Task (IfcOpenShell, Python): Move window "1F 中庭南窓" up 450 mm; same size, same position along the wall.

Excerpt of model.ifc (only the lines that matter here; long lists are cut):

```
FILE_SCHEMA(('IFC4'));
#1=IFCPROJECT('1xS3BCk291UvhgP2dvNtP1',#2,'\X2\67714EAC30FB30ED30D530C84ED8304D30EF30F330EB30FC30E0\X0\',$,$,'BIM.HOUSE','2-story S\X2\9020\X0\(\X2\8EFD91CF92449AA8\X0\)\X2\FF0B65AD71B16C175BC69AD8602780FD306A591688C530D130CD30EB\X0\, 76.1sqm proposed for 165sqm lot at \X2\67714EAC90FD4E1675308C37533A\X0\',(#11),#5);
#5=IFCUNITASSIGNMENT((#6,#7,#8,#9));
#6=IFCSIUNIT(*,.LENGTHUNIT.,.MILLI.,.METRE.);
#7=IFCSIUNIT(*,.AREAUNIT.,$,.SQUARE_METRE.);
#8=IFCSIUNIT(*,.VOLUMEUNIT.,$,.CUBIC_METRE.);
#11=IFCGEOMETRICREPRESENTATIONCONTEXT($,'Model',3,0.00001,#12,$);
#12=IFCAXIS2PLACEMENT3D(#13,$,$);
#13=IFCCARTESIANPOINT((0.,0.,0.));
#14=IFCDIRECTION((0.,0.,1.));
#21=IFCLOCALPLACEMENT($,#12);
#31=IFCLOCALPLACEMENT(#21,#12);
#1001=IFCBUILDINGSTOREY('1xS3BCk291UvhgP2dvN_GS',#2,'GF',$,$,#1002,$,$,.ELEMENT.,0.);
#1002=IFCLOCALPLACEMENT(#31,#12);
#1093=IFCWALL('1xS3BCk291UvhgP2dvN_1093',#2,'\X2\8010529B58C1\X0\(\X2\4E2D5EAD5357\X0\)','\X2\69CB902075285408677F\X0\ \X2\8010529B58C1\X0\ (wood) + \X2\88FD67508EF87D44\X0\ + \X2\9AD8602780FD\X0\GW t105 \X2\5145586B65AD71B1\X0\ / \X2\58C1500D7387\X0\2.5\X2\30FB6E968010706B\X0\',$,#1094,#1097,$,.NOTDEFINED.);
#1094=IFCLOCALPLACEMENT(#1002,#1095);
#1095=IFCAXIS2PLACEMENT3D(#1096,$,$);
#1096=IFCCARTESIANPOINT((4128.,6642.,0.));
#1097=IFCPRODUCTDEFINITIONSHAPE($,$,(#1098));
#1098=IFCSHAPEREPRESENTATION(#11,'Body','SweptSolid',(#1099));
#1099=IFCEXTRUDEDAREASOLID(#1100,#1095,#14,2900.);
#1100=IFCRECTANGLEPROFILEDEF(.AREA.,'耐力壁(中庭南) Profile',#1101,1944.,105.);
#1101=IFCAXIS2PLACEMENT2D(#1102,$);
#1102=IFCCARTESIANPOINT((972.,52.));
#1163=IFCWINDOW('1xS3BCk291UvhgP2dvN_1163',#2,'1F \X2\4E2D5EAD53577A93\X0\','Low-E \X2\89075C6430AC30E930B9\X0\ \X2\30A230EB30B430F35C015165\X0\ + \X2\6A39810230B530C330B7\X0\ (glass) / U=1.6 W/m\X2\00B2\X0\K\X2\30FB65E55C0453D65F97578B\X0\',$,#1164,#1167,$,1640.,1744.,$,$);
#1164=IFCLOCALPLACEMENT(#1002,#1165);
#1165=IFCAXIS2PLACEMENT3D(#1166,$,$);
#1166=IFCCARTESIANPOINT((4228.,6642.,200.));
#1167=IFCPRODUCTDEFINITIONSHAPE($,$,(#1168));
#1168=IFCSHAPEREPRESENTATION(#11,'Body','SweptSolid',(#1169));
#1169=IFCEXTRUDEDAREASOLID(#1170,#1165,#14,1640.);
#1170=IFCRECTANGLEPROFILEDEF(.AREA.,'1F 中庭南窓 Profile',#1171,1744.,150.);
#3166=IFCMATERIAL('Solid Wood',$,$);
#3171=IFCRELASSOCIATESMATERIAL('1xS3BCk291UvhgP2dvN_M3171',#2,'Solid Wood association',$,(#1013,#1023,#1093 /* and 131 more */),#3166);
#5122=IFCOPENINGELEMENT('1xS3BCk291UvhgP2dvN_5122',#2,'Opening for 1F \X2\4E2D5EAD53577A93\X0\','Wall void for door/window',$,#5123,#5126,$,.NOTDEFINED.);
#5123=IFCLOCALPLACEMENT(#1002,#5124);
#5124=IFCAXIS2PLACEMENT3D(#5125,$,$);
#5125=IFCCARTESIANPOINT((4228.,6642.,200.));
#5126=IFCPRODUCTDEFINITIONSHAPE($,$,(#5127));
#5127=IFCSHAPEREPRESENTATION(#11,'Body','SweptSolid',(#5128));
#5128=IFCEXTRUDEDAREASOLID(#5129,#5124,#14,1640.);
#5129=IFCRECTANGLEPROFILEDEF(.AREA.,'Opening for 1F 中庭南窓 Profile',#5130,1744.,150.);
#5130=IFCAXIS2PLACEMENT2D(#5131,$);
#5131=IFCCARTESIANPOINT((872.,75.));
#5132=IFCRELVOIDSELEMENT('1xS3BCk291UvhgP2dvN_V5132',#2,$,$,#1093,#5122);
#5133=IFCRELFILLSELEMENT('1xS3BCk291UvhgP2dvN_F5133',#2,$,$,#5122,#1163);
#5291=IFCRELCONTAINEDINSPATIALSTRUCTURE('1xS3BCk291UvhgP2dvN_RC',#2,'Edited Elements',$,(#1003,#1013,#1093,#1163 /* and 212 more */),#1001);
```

```python
import numpy as np
import ifcopenshell
import ifcopenshell.api.geometry
import ifcopenshell.util.placement
import ifcopenshell.util.unit

model = ifcopenshell.open("model.ifc")
unit_scale = ifcopenshell.util.unit.calculate_unit_scale(model)

window = model.by_id(1163)
opening = window.FillsVoids[0].RelatingOpeningElement
dz = 450.0

shift = np.array([0.0, 0.0, dz])
# The window is not placed relative to its opening, so move both.
for product in (opening, window):
    matrix = ifcopenshell.util.placement.get_local_placement(product.ObjectPlacement)
    matrix[:3, 3] += shift
    ifcopenshell.api.geometry.edit_object_placement(model, product=product, matrix=matrix, is_si=False)

print(f"moved by {dz * unit_scale:+.3f} m")

model.write("model-out.ifc")
```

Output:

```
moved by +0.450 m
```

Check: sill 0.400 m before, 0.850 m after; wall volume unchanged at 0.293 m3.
